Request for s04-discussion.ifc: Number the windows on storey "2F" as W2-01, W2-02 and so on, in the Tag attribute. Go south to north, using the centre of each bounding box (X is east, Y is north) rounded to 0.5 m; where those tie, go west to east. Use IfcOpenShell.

First a look at what the model holds.

```python
import ifcopenshell
import ifcopenshell.util.element
import ifcopenshell.util.placement

model = ifcopenshell.open("s04-discussion.ifc")
print(model.schema)
storey = next(s for s in model.by_type("IfcBuildingStorey") if s.Name == "2F")
windows = [e for e in ifcopenshell.util.element.get_decomposition(storey) if e.is_a("IfcWindow")]
for e in sorted(windows, key=lambda e: e.id()):
    origin = ifcopenshell.util.placement.get_local_placement(e.ObjectPlacement)[:3, 3]
    print(e.id(), e.Tag, e.Name, origin.round(2) + 0.0, sep=" | ")
```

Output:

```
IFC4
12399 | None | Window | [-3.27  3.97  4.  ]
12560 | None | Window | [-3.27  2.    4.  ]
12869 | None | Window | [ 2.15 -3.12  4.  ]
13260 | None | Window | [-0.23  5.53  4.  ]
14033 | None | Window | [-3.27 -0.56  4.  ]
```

```python
import ifcopenshell
import ifcopenshell.geom
import ifcopenshell.util.element
import ifcopenshell.util.shape

model = ifcopenshell.open("s04-discussion.ifc")
settings = ifcopenshell.geom.settings()
settings.set("use-world-coords", True)


def centre(element):
    shape = ifcopenshell.geom.create_shape(settings, element)
    return ifcopenshell.util.shape.get_bbox_centroid(shape.geometry)


storey = next(s for s in model.by_type("IfcBuildingStorey") if s.Name == "2F")
windows = [e for e in ifcopenshell.util.element.get_decomposition(storey) if e.is_a("IfcWindow")]

# Insertion points can sit at a corner or the storey origin, so sort by the geometry (in metres).
centres = {e: centre(e) for e in windows}
windows.sort(key=lambda e: (round(centres[e][1] / 0.5), centres[e][0]))

for i, e in enumerate(windows, start=1):
    number = f"W2-{i:02d}"
    e.Tag = number
    print(e.id(), number)

model.write("s04-discussion-out.ifc")
```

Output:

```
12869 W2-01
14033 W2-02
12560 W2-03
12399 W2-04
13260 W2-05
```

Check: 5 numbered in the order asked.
